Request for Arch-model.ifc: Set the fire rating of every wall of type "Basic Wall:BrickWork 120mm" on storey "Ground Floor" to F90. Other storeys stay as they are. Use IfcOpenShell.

First a look at what the model holds.

```python
import ifcopenshell
import ifcopenshell.util.element

model = ifcopenshell.open("Arch-model.ifc")
print(model.schema)
storey = next(s for s in model.by_type("IfcBuildingStorey") if s.Name == "Ground Floor")
walls = [e for e in ifcopenshell.util.element.get_decomposition(storey) if e.is_a("IfcWall")]
seen = {}
for e in walls:
    element_type = ifcopenshell.util.element.get_type(e)
    key = (element_type.Name if element_type != e and element_type else None, ifcopenshell.util.element.get_pset(e, "Pset_WallCommon", "FireRating"))
    seen[key] = seen.get(key, 0) + 1
for (name, value), count in sorted(seen.items(), key=str):
    print(count, "x", name, "|", value)
```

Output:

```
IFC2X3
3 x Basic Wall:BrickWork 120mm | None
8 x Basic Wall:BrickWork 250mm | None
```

```python
import ifcopenshell
import ifcopenshell.api.pset
import ifcopenshell.util.element

model = ifcopenshell.open("Arch-model.ifc")

storey = next(s for s in model.by_type("IfcBuildingStorey") if s.Name == "Ground Floor")
walls = [e for e in ifcopenshell.util.element.get_decomposition(storey) if e.is_a("IfcWall")]

count = 0
for e in walls:
    element_type = ifcopenshell.util.element.get_type(e)
    if element_type in (None, e) or element_type.Name != "Basic Wall:BrickWork 120mm":
        continue
    # add_pset returns the element's existing set when there is one.
    pset = ifcopenshell.api.pset.add_pset(model, product=e, name="Pset_WallCommon")
    ifcopenshell.api.pset.edit_pset(model, pset=pset, properties={"FireRating": "F90"})
    count += 1

print(count, "walls updated")

model.write("Arch-model-out.ifc")
```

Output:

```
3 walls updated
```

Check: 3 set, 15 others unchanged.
